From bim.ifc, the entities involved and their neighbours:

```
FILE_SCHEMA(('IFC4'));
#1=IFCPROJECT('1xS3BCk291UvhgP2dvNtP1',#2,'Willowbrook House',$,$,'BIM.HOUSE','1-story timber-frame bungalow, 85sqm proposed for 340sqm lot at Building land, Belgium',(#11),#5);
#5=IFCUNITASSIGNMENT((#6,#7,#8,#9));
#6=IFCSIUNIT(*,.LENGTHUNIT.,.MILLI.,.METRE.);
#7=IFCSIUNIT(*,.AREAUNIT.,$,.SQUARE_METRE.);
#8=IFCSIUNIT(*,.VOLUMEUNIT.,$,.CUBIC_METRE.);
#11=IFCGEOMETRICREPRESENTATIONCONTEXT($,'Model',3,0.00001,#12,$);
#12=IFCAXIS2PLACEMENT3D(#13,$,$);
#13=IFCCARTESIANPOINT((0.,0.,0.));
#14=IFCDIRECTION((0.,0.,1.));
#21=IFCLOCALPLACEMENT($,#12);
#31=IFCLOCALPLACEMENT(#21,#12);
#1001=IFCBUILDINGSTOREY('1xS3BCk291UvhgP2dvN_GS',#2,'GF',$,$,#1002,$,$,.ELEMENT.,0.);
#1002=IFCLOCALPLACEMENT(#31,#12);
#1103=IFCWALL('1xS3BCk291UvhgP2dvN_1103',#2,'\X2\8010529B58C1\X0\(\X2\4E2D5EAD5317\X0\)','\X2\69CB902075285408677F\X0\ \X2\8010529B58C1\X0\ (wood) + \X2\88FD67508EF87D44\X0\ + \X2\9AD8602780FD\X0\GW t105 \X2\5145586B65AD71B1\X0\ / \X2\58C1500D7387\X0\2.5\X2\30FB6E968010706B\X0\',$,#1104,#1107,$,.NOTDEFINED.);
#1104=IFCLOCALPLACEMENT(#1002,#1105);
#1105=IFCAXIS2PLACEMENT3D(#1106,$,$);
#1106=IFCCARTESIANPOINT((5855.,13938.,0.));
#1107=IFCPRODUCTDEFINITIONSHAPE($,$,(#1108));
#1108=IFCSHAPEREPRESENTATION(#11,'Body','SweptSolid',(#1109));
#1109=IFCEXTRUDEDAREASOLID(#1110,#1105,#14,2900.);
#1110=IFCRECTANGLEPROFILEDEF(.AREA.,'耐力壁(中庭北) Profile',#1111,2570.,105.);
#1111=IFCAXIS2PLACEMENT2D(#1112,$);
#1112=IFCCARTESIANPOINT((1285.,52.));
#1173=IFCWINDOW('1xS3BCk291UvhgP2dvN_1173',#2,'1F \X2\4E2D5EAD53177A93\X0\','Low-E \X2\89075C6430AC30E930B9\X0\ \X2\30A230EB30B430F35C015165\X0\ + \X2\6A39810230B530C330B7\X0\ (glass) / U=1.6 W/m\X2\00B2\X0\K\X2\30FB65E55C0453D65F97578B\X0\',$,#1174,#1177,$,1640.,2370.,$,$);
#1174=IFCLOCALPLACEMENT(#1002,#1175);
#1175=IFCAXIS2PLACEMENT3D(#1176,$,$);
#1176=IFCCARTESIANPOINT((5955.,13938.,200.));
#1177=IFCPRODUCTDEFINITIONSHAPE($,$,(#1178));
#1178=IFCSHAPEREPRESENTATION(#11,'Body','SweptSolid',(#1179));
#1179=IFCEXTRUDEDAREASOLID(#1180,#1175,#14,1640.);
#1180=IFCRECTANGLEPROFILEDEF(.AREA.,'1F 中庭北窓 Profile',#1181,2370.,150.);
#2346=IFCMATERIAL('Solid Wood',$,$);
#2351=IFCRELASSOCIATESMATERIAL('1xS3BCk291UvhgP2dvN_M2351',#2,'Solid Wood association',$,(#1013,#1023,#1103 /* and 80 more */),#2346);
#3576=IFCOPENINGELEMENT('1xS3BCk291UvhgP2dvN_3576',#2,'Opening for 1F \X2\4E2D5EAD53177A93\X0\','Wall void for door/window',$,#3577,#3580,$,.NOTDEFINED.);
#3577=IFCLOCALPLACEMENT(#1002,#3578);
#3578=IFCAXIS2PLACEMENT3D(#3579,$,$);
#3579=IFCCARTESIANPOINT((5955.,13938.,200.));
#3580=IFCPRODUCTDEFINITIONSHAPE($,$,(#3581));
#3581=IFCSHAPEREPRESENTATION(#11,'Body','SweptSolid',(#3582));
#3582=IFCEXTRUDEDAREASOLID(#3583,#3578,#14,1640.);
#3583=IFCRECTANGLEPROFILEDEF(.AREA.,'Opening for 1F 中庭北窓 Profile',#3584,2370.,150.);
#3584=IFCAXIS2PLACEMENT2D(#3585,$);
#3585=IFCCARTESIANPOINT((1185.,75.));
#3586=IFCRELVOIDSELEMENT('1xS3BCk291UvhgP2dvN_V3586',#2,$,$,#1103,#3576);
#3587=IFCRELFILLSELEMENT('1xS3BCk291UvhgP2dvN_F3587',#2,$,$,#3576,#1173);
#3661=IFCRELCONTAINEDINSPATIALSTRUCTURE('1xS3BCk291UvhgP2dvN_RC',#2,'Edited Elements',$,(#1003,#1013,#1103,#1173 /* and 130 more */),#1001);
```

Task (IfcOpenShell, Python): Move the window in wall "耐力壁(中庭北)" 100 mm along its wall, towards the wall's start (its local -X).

```python
import ifcopenshell
import ifcopenshell.api.geometry
import ifcopenshell.util.placement
import ifcopenshell.util.unit

model = ifcopenshell.open("bim.ifc")
unit_scale = ifcopenshell.util.unit.calculate_unit_scale(model)

window = model.by_guid("1xS3BCk291UvhgP2dvN_1173")
opening = window.FillsVoids[0].RelatingOpeningElement
wall = opening.VoidsElements[0].RelatingBuildingElement

wall_matrix = ifcopenshell.util.placement.get_local_placement(wall.ObjectPlacement)
shift = wall_matrix[:3, 0] * -0.1 / unit_scale
before = ifcopenshell.util.placement.get_local_placement(window.ObjectPlacement)[:3, 3].copy()

# The window is not placed relative to its opening, so move both.
for product in (opening, window):
    matrix = ifcopenshell.util.placement.get_local_placement(product.ObjectPlacement)
    matrix[:3, 3] += shift
    ifcopenshell.api.geometry.edit_object_placement(model, product=product, matrix=matrix, is_si=False)

after = ifcopenshell.util.placement.get_local_placement(window.ObjectPlacement)[:3, 3]
print("window moved by", (after - before).round(3) + 0.0)

model.write("bim_rev.ifc")
```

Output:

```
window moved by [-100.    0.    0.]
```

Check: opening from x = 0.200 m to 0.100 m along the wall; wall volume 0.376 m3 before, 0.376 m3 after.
